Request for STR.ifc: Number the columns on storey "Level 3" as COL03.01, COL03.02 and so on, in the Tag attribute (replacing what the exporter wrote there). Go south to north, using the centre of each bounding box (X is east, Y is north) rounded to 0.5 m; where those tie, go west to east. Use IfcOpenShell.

First a look at what the model holds.

```python
import ifcopenshell
import ifcopenshell.util.element
import ifcopenshell.util.placement

model = ifcopenshell.open("STR.ifc")
print(model.schema)
storey = next(s for s in model.by_type("IfcBuildingStorey") if s.Name == "Level 3")
columns = [e for e in ifcopenshell.util.element.get_decomposition(storey) if e.is_a("IfcColumn")]
for e in sorted(columns, key=lambda e: e.id()):
    origin = ifcopenshell.util.placement.get_local_placement(e.ObjectPlacement)[:3, 3]
    print(e.id(), e.Tag, e.Name, origin.round(2) + 0.0, sep=" | ")
```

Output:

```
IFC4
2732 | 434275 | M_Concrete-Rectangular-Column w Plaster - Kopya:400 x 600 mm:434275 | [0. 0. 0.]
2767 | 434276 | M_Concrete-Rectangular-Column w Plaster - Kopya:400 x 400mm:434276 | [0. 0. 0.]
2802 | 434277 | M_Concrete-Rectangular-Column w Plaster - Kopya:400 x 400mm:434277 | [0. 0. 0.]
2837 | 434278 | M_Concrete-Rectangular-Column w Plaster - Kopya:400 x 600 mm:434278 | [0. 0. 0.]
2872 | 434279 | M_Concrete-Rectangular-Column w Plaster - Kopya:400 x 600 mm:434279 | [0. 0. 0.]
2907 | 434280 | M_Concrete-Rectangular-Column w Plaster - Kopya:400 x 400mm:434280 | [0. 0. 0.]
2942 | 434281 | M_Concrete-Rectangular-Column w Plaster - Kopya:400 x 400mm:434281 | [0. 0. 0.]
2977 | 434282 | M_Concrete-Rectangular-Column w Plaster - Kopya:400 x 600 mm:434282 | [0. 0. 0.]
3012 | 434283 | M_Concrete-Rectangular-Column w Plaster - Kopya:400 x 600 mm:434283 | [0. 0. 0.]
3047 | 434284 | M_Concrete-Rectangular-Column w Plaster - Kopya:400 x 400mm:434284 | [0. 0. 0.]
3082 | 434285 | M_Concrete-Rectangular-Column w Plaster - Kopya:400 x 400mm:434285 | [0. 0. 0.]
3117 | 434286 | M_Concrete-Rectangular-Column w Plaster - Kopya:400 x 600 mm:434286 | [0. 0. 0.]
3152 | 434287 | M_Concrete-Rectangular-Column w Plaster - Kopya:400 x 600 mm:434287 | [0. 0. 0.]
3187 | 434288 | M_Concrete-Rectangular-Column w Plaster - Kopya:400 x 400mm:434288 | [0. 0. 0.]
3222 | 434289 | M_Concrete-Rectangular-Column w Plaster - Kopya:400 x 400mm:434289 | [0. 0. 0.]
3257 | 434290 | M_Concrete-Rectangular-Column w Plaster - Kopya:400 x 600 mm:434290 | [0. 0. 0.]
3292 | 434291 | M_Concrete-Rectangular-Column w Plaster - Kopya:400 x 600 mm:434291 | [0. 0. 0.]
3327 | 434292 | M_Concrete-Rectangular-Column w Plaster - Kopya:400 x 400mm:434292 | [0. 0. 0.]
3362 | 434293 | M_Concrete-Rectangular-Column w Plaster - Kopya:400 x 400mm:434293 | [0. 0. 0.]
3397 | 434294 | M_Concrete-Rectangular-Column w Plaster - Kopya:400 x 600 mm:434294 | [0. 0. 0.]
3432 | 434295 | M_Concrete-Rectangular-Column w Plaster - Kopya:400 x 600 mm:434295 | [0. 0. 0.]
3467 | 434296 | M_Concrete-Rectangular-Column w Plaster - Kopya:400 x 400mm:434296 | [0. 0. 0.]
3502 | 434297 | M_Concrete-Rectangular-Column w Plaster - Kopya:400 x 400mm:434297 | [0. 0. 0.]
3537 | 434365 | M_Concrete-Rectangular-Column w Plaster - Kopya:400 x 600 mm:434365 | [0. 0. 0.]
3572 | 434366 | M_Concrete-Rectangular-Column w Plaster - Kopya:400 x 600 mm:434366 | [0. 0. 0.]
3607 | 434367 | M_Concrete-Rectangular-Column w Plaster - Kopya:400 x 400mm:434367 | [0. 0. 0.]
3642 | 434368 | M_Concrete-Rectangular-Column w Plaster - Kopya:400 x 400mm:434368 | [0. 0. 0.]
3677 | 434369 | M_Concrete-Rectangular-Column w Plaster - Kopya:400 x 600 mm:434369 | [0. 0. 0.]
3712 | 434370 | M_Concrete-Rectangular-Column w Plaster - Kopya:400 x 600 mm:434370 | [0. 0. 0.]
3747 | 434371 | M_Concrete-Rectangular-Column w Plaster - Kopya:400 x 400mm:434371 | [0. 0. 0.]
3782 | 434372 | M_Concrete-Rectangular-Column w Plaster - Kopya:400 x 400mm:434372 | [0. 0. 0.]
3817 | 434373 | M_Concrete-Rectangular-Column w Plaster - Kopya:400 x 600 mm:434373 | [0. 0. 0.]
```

```python
import ifcopenshell
import ifcopenshell.geom
import ifcopenshell.util.element
import ifcopenshell.util.shape

model = ifcopenshell.open("STR.ifc")
settings = ifcopenshell.geom.settings()
settings.set("use-world-coords", True)


def centre(element):
    shape = ifcopenshell.geom.create_shape(settings, element)
    return ifcopenshell.util.shape.get_bbox_centroid(shape.geometry)


storey = next(s for s in model.by_type("IfcBuildingStorey") if s.Name == "Level 3")
columns = [e for e in ifcopenshell.util.element.get_decomposition(storey) if e.is_a("IfcColumn")]

# Insertion points can sit at a corner or the storey origin, so sort by the geometry (in metres).
centres = {e: centre(e) for e in columns}
columns.sort(key=lambda e: (round(centres[e][1] / 0.5), centres[e][0]))

for i, e in enumerate(columns, start=1):
    number = f"COL03.{i:02d}"
    e.Tag = number
    print(e.id(), number)

model.write("STR_updated.ifc")
```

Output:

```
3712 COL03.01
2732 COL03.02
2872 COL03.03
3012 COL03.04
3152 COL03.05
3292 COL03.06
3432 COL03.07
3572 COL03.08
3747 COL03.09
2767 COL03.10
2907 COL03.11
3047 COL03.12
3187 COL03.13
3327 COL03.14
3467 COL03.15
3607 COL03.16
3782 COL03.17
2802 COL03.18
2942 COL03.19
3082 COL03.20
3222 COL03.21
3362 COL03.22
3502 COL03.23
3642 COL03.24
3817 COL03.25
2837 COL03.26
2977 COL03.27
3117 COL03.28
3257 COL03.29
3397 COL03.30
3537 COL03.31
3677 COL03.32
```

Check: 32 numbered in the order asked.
